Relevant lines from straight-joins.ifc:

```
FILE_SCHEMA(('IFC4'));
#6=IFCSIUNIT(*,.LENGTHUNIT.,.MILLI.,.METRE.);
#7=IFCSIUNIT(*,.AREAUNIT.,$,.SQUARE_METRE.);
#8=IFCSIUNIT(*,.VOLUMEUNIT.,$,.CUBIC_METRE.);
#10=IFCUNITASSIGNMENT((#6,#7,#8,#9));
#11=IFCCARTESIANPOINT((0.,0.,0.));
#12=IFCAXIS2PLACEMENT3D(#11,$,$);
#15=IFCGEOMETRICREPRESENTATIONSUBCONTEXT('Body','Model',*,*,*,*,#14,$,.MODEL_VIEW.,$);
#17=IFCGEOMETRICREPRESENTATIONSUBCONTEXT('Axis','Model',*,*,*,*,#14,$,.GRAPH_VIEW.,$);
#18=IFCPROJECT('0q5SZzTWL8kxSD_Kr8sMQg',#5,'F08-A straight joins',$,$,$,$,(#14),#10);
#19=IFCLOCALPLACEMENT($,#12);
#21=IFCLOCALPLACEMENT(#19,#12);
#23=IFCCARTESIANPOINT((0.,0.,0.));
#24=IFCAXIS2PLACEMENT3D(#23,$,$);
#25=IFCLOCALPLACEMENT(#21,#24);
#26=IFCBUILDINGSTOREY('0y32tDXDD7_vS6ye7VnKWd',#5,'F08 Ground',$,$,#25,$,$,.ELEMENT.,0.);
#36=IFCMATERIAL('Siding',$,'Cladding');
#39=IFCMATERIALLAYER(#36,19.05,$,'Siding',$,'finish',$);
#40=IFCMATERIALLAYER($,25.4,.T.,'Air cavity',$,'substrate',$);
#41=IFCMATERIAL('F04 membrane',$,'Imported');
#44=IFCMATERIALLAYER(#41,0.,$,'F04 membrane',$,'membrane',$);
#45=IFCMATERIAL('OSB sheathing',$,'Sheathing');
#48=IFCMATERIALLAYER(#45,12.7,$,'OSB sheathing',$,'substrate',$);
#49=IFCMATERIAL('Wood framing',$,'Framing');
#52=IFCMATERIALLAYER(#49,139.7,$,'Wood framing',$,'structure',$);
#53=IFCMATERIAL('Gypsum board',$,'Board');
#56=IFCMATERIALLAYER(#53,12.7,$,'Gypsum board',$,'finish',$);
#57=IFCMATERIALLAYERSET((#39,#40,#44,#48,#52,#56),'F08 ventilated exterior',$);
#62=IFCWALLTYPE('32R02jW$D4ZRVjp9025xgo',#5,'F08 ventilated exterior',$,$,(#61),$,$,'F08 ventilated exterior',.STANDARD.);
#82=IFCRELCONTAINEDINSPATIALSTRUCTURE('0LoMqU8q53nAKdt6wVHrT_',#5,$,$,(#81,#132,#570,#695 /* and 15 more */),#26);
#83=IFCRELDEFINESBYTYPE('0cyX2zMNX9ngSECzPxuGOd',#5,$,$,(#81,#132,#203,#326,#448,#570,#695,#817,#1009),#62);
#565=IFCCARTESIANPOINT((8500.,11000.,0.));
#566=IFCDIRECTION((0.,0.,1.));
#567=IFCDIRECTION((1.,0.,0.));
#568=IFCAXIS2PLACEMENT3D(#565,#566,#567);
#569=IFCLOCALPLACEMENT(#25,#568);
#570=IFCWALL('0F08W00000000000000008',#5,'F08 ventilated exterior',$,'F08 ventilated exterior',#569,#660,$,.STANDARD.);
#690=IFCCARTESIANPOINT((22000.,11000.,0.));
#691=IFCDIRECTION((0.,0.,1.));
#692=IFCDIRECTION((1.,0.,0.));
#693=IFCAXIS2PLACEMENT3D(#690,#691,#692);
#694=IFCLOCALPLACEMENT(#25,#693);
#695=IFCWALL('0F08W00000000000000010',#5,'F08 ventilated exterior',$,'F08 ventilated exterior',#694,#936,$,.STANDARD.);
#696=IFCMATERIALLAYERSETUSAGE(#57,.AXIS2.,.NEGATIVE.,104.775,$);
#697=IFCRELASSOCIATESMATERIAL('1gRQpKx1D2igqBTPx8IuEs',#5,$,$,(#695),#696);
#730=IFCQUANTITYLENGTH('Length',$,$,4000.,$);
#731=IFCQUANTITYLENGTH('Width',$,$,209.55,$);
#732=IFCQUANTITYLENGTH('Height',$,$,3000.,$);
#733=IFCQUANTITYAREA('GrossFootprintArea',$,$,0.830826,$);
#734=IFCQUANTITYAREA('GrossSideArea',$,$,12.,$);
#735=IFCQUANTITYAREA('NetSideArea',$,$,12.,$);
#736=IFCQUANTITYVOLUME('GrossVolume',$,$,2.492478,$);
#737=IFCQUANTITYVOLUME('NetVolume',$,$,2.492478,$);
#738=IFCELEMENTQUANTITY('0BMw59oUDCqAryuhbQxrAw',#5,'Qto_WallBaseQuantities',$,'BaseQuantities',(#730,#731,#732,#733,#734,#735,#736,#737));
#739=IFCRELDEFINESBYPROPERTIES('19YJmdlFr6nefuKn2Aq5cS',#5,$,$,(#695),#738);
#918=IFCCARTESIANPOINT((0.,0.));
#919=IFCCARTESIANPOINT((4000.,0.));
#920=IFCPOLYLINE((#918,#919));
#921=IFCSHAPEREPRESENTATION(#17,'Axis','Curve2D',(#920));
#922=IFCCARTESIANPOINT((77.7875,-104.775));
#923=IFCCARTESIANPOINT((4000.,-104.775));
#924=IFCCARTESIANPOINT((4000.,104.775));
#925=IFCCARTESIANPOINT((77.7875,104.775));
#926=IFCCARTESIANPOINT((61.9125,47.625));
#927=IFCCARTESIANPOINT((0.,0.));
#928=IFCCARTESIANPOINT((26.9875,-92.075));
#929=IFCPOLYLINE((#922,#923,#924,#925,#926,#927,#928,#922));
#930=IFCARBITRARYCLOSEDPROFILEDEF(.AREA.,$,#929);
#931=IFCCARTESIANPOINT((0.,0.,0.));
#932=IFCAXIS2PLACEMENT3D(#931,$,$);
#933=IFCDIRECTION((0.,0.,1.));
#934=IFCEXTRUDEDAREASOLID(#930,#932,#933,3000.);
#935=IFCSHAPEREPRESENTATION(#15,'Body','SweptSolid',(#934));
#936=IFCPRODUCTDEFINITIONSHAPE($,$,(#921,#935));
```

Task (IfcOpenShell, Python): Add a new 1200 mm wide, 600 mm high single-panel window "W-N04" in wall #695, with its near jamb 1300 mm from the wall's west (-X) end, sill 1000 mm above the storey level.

```python
import numpy as np
import ifcopenshell
import ifcopenshell.api.feature
import ifcopenshell.api.geometry
import ifcopenshell.api.pset
import ifcopenshell.api.root
import ifcopenshell.api.spatial
import ifcopenshell.geom
import ifcopenshell.util.element
import ifcopenshell.util.placement
import ifcopenshell.util.representation
import ifcopenshell.util.shape
import ifcopenshell.util.unit

model = ifcopenshell.open("straight-joins.ifc")
unit_scale = ifcopenshell.util.unit.calculate_unit_scale(model)
area_scale = ifcopenshell.util.unit.calculate_unit_scale(model, "AREAUNIT")
volume_scale = ifcopenshell.util.unit.calculate_unit_scale(model, "VOLUMEUNIT")
settings = ifcopenshell.geom.settings()


def volume(element):
    """Net volume in cubic metres, openings subtracted."""
    shape = ifcopenshell.geom.create_shape(settings, element)
    return ifcopenshell.util.shape.get_volume(shape.geometry)


wall = model.by_id(695)
storey = ifcopenshell.util.element.get_container(wall, ifc_class="IfcBuildingStorey")
context = ifcopenshell.util.representation.get_context(model, "Model", "Body", "MODEL_VIEW")
before = volume(wall)

width, height, from_end, sill = 1.2, 0.6, 1.3, 1  # metres

# The wall runs along its own X axis, and the end named is its -X end.
wall_shape = ifcopenshell.geom.create_shape(settings, wall)
x, y, z = ifcopenshell.util.shape.get_vertices(wall_shape.geometry).T
start = x.min() + from_end
face, thickness = float(y.min()), float(y.max() - y.min())
wall_matrix = ifcopenshell.util.placement.get_local_placement(wall.ObjectPlacement)
level = ifcopenshell.util.placement.get_local_placement(storey.ObjectPlacement)[2, 3]


def in_wall(x, y):
    """Placement at x, y metres in the wall's axes, at sill height."""
    matrix = wall_matrix.copy()
    matrix[:, 3] = wall_matrix @ np.array([x / unit_scale, y / unit_scale, 0.0, 1.0])
    matrix[2, 3] = level + sill / unit_scale
    return matrix


# Opening: a box that overshoots both wall faces by 50 mm.
opening = ifcopenshell.api.root.create_entity(model, ifc_class="IfcOpeningElement", predefined_type="OPENING")
box = ifcopenshell.api.geometry.add_wall_representation(
    model, context=context, length=width, height=height, thickness=thickness + 0.1
)
ifcopenshell.api.geometry.assign_representation(model, product=opening, representation=box)
ifcopenshell.api.geometry.edit_object_placement(model, product=opening, matrix=in_wall(start, face - 0.05), is_si=False)
ifcopenshell.api.feature.add_feature(model, feature=opening, element=wall)

window = ifcopenshell.api.root.create_entity(model, ifc_class="IfcWindow", name="W-N04", predefined_type="WINDOW")
window.OverallWidth, window.OverallHeight = width / unit_scale, height / unit_scale
window.PartitioningType = "SINGLE_PANEL"
body = ifcopenshell.api.geometry.add_window_representation(
    model,
    context=context,
    overall_width=window.OverallWidth,
    overall_height=window.OverallHeight,
    partition_type="SINGLE_PANEL",
)
ifcopenshell.api.geometry.assign_representation(model, product=window, representation=body)
ifcopenshell.api.spatial.assign_container(model, products=[window], relating_structure=storey)
ifcopenshell.api.feature.add_filling(model, opening=opening, element=window)

# Centre the window in the wall's thickness.
ifcopenshell.api.geometry.edit_object_placement(model, product=window, matrix=in_wall(start, face), is_si=False)
window_shape = ifcopenshell.geom.create_shape(settings, window)
depth = ifcopenshell.util.shape.get_vertices(window_shape.geometry)[:, 1]
offset = face + thickness / 2 - (depth.min() + depth.max()) / 2
ifcopenshell.api.geometry.edit_object_placement(model, product=window, matrix=in_wall(start, offset), is_si=False)

after = volume(wall)

# Update the wall's stored quantities.
qto = model.by_id(ifcopenshell.util.element.get_pset(wall, "Qto_WallBaseQuantities", should_inherit=False)["id"])
ifcopenshell.api.pset.edit_qto(model, qto=qto, properties={
    "NetSideArea": after / thickness / area_scale,
    "NetVolume": after / volume_scale,
})

print(f"wall volume {before:.3f} -> {after:.3f} m3")

model.write("straight-joins_updated.ifc")
```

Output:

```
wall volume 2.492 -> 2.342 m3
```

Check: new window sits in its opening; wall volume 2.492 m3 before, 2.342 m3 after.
